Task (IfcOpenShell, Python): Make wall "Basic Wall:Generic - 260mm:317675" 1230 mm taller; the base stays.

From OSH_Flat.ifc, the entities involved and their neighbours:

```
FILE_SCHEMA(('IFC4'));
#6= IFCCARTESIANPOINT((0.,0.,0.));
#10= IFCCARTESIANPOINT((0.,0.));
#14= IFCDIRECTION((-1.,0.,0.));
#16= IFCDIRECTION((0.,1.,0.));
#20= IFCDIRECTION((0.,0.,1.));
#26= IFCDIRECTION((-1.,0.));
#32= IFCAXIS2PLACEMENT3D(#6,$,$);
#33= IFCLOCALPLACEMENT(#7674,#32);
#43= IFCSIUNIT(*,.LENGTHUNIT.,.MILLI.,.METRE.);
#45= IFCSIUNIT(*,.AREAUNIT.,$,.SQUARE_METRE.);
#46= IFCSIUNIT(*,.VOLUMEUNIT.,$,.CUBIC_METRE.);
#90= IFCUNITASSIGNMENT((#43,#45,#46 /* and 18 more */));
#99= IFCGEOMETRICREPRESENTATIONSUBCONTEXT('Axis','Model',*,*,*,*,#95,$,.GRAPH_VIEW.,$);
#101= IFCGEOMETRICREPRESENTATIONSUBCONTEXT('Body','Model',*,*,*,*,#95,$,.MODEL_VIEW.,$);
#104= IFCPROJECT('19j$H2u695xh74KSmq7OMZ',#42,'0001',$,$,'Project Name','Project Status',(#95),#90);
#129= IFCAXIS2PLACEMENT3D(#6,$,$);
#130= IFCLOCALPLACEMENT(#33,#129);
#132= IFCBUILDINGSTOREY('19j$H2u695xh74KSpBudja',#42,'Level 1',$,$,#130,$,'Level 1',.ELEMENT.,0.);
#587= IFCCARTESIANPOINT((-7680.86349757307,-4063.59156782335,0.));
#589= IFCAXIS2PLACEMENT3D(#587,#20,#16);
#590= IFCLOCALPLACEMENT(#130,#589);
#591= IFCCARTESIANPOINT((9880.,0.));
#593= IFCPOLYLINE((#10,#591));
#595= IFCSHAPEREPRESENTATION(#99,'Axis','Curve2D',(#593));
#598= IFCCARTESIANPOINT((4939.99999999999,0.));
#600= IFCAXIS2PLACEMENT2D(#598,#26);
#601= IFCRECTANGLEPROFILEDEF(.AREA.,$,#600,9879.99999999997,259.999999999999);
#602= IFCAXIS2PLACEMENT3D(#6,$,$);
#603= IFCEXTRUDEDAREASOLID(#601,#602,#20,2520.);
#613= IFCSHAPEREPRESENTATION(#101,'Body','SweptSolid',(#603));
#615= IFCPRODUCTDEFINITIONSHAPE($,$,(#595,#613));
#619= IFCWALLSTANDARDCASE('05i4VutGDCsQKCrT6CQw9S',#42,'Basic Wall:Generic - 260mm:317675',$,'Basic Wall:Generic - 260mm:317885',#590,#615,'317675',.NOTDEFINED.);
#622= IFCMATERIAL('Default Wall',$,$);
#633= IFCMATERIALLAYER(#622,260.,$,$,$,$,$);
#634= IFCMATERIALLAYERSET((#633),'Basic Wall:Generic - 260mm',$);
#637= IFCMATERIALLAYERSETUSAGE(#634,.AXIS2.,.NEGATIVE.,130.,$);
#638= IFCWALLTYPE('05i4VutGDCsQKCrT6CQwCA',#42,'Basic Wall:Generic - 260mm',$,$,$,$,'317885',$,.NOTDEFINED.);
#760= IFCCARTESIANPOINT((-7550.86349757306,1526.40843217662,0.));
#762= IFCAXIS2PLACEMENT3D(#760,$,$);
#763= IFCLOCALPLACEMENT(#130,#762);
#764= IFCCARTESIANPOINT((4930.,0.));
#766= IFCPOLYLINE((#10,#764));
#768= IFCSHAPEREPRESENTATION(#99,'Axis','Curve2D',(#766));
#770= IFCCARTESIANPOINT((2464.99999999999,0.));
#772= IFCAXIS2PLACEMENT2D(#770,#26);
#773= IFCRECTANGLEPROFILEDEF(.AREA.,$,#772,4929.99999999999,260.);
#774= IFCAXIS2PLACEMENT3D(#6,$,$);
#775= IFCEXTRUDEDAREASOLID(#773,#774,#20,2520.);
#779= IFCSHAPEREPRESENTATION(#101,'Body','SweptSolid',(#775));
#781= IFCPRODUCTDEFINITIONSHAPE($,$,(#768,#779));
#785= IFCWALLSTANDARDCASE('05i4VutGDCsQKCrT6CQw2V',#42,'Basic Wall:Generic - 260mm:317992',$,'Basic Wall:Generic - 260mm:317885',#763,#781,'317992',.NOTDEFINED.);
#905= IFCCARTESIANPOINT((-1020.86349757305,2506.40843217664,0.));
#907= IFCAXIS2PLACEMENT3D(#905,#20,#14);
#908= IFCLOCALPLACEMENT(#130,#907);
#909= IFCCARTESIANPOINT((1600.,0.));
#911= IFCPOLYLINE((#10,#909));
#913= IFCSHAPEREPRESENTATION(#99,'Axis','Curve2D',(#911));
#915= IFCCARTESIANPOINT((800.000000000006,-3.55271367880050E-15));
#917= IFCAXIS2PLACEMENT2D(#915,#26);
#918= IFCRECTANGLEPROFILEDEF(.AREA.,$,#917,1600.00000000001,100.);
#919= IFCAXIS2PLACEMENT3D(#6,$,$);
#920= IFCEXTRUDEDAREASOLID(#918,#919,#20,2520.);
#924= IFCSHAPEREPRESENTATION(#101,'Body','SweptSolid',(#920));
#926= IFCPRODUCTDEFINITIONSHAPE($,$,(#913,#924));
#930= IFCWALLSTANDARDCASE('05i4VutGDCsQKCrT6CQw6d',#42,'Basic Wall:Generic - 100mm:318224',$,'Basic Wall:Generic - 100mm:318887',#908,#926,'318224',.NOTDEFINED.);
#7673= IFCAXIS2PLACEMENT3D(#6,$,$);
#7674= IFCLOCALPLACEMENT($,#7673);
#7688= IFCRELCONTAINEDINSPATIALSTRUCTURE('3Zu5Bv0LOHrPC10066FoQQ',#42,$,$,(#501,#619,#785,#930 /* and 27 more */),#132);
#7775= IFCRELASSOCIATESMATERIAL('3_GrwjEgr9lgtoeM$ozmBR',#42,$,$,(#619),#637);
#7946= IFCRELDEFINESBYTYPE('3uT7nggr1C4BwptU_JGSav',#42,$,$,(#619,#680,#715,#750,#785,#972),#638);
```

```python
import ifcopenshell
import ifcopenshell.geom
import ifcopenshell.util.representation
import ifcopenshell.util.shape

model = ifcopenshell.open("OSH_Flat.ifc")
settings = ifcopenshell.geom.settings()


def volume(element):
    """Net volume in cubic metres, openings subtracted."""
    shape = ifcopenshell.geom.create_shape(settings, element)
    return ifcopenshell.util.shape.get_volume(shape.geometry)


wall = model.by_guid("05i4VutGDCsQKCrT6CQw9S")
before = volume(wall)

body = ifcopenshell.util.representation.get_representation(wall, "Model", "Body")
solid = body.Items[0]
old_height = solid.Depth
solid.Depth += 1230.0
after = volume(wall)

print(f"height {old_height:g} -> {solid.Depth:g}, volume {before:.3f} -> {after:.3f} m3")

model.write("OSH_Flat_v2.ifc")
```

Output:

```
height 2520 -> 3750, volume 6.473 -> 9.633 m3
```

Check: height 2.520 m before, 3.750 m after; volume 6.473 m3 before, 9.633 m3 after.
